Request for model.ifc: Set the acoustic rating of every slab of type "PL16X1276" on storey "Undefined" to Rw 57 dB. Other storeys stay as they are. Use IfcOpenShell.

First a look at what the model holds.

```python
import ifcopenshell
import ifcopenshell.util.element

model = ifcopenshell.open("model.ifc")
print(model.schema)
storey = next(s for s in model.by_type("IfcBuildingStorey") if s.Name == "Undefined")
slabs = [e for e in ifcopenshell.util.element.get_decomposition(storey) if e.is_a("IfcSlab")]
seen = {}
for e in slabs:
    element_type = ifcopenshell.util.element.get_type(e)
    key = (element_type.Name if element_type != e and element_type else None, ifcopenshell.util.element.get_pset(e, "Pset_SlabCommon", "AcousticRating"))
    seen[key] = seen.get(key, 0) + 1
for (name, value), count in sorted(seen.items(), key=str):
    print(count, "x", name, "|", value)
```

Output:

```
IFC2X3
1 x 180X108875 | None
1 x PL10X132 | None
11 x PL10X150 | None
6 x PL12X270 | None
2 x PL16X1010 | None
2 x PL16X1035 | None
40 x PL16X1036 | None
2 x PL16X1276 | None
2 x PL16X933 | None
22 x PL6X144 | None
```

```python
import ifcopenshell
import ifcopenshell.api.pset
import ifcopenshell.util.element

model = ifcopenshell.open("model.ifc")

storey = next(s for s in model.by_type("IfcBuildingStorey") if s.Name == "Undefined")
slabs = [e for e in ifcopenshell.util.element.get_decomposition(storey) if e.is_a("IfcSlab")]

count = 0
for e in slabs:
    element_type = ifcopenshell.util.element.get_type(e)
    if element_type in (None, e) or element_type.Name != "PL16X1276":
        continue
    # add_pset returns the element's existing set when there is one.
    pset = ifcopenshell.api.pset.add_pset(model, product=e, name="Pset_SlabCommon")
    ifcopenshell.api.pset.edit_pset(model, pset=pset, properties={"AcousticRating": "Rw 57 dB"})
    count += 1

print(count, "slabs updated")

model.write("model_rev.ifc")
```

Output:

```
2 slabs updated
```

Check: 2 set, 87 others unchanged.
